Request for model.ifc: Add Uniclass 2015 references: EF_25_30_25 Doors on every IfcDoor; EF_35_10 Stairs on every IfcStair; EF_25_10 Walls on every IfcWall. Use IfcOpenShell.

First a look at what the model holds.

```python
import ifcopenshell

model = ifcopenshell.open("model.ifc")
print(model.schema)
print("classifications:", [c.Name for c in model.by_type("IfcClassification")])
for ifc_class in ("IfcDoor", "IfcRoof", "IfcStair", "IfcWall", "IfcWindow"):
    print(ifc_class, len(model.by_type(ifc_class)))
```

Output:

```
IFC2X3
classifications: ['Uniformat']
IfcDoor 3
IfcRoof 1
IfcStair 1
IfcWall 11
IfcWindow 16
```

```python
import ifcopenshell
import ifcopenshell.api.classification

model = ifcopenshell.open("model.ifc")

# IFC2X3 requires Source and Edition and has no link from the project to the system.
system = model.create_entity("IfcClassification", Source="NBS", Edition="2015", Name="Uniclass 2015")

codes = {
    "IfcDoor": ("EF_25_30_25", "Doors"),
    "IfcStair": ("EF_35_10", "Stairs"),
    "IfcWall": ("EF_25_10", "Walls"),
}
for ifc_class, (code, name) in codes.items():
    products = model.by_type(ifc_class)
    ifcopenshell.api.classification.add_reference(
        model, products=products, classification=system, identification=code, name=name
    )
    print(code, len(products))

model.write("model_updated.ifc")
```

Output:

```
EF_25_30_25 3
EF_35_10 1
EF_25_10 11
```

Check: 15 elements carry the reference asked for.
